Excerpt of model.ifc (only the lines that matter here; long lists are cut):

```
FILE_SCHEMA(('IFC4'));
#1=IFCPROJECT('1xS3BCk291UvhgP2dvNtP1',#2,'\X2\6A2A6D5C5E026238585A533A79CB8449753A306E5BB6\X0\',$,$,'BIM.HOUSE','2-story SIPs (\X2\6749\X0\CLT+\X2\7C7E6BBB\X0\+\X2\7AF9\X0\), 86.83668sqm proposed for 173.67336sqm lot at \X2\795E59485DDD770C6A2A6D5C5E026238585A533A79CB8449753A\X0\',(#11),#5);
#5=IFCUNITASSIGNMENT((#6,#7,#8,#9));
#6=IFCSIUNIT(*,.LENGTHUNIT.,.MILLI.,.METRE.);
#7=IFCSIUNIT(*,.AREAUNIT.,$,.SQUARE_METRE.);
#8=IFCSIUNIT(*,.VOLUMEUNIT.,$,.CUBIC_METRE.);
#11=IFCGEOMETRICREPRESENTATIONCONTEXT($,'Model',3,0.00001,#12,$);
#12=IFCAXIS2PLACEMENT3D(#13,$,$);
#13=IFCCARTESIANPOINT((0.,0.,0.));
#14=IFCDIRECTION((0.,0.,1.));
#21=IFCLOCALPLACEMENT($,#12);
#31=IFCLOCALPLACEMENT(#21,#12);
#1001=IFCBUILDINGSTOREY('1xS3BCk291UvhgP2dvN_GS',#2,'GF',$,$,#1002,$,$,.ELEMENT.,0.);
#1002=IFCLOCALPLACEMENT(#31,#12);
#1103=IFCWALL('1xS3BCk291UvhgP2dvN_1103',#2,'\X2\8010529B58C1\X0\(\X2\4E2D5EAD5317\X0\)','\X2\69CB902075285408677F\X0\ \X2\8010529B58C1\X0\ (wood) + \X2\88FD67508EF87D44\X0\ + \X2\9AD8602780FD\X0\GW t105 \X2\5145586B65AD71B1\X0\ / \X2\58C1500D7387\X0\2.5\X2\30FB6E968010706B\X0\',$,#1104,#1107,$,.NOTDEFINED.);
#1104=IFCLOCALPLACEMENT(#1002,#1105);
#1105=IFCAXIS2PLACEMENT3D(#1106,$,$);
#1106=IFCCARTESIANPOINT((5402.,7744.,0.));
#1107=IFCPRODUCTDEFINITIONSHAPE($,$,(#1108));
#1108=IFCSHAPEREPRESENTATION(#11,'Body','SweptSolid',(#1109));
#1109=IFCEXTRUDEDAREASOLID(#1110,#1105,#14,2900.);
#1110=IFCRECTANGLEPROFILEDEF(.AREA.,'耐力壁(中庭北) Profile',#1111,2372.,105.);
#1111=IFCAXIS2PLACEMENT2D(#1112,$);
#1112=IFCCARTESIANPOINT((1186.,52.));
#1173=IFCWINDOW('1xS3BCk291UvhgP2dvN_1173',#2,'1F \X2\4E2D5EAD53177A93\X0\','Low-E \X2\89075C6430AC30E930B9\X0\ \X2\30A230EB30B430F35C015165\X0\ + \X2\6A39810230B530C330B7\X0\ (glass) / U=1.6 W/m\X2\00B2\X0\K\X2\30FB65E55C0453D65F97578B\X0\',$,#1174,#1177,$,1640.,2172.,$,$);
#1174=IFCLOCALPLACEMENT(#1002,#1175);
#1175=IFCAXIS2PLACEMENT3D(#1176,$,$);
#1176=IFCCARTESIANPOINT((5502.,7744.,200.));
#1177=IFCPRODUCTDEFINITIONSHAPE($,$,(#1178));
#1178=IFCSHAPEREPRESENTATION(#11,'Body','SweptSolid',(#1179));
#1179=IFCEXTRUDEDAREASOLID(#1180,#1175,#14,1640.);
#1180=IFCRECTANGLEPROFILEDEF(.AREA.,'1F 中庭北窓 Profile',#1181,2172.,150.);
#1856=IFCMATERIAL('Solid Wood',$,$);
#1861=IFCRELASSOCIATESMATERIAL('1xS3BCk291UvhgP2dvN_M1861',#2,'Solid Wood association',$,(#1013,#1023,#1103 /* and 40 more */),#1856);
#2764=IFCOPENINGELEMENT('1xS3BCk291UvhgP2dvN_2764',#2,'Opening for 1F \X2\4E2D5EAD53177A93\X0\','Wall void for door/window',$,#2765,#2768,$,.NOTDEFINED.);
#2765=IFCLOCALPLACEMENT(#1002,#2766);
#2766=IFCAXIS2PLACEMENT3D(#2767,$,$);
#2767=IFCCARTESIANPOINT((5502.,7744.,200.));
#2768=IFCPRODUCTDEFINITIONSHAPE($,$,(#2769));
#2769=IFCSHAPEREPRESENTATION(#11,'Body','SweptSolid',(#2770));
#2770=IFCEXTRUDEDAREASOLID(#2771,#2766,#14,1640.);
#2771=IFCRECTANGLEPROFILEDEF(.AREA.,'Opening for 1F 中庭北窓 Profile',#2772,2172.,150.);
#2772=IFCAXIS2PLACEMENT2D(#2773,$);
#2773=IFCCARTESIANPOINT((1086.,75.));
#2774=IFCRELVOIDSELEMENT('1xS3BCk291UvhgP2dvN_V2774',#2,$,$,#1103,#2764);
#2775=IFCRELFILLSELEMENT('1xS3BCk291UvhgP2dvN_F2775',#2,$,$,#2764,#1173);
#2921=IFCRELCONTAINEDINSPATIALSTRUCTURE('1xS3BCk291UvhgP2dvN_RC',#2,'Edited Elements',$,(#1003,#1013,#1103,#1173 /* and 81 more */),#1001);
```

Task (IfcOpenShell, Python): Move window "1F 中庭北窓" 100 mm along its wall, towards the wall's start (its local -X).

```python
import ifcopenshell
import ifcopenshell.api.geometry
import ifcopenshell.util.placement
import ifcopenshell.util.unit

model = ifcopenshell.open("model.ifc")
unit_scale = ifcopenshell.util.unit.calculate_unit_scale(model)

window = model.by_guid("1xS3BCk291UvhgP2dvN_1173")
opening = window.FillsVoids[0].RelatingOpeningElement
wall = opening.VoidsElements[0].RelatingBuildingElement

wall_matrix = ifcopenshell.util.placement.get_local_placement(wall.ObjectPlacement)
shift = wall_matrix[:3, 0] * -0.1 / unit_scale
before = ifcopenshell.util.placement.get_local_placement(window.ObjectPlacement)[:3, 3].copy()

# The window is not placed relative to its opening, so move both.
for product in (opening, window):
    matrix = ifcopenshell.util.placement.get_local_placement(product.ObjectPlacement)
    matrix[:3, 3] += shift
    ifcopenshell.api.geometry.edit_object_placement(model, product=product, matrix=matrix, is_si=False)

after = ifcopenshell.util.placement.get_local_placement(window.ObjectPlacement)[:3, 3]
print("window moved by", (after - before).round(3) + 0.0)

model.write("model_updated.ifc")
```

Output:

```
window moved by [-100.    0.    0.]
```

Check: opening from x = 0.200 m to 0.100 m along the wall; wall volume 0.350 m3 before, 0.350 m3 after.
